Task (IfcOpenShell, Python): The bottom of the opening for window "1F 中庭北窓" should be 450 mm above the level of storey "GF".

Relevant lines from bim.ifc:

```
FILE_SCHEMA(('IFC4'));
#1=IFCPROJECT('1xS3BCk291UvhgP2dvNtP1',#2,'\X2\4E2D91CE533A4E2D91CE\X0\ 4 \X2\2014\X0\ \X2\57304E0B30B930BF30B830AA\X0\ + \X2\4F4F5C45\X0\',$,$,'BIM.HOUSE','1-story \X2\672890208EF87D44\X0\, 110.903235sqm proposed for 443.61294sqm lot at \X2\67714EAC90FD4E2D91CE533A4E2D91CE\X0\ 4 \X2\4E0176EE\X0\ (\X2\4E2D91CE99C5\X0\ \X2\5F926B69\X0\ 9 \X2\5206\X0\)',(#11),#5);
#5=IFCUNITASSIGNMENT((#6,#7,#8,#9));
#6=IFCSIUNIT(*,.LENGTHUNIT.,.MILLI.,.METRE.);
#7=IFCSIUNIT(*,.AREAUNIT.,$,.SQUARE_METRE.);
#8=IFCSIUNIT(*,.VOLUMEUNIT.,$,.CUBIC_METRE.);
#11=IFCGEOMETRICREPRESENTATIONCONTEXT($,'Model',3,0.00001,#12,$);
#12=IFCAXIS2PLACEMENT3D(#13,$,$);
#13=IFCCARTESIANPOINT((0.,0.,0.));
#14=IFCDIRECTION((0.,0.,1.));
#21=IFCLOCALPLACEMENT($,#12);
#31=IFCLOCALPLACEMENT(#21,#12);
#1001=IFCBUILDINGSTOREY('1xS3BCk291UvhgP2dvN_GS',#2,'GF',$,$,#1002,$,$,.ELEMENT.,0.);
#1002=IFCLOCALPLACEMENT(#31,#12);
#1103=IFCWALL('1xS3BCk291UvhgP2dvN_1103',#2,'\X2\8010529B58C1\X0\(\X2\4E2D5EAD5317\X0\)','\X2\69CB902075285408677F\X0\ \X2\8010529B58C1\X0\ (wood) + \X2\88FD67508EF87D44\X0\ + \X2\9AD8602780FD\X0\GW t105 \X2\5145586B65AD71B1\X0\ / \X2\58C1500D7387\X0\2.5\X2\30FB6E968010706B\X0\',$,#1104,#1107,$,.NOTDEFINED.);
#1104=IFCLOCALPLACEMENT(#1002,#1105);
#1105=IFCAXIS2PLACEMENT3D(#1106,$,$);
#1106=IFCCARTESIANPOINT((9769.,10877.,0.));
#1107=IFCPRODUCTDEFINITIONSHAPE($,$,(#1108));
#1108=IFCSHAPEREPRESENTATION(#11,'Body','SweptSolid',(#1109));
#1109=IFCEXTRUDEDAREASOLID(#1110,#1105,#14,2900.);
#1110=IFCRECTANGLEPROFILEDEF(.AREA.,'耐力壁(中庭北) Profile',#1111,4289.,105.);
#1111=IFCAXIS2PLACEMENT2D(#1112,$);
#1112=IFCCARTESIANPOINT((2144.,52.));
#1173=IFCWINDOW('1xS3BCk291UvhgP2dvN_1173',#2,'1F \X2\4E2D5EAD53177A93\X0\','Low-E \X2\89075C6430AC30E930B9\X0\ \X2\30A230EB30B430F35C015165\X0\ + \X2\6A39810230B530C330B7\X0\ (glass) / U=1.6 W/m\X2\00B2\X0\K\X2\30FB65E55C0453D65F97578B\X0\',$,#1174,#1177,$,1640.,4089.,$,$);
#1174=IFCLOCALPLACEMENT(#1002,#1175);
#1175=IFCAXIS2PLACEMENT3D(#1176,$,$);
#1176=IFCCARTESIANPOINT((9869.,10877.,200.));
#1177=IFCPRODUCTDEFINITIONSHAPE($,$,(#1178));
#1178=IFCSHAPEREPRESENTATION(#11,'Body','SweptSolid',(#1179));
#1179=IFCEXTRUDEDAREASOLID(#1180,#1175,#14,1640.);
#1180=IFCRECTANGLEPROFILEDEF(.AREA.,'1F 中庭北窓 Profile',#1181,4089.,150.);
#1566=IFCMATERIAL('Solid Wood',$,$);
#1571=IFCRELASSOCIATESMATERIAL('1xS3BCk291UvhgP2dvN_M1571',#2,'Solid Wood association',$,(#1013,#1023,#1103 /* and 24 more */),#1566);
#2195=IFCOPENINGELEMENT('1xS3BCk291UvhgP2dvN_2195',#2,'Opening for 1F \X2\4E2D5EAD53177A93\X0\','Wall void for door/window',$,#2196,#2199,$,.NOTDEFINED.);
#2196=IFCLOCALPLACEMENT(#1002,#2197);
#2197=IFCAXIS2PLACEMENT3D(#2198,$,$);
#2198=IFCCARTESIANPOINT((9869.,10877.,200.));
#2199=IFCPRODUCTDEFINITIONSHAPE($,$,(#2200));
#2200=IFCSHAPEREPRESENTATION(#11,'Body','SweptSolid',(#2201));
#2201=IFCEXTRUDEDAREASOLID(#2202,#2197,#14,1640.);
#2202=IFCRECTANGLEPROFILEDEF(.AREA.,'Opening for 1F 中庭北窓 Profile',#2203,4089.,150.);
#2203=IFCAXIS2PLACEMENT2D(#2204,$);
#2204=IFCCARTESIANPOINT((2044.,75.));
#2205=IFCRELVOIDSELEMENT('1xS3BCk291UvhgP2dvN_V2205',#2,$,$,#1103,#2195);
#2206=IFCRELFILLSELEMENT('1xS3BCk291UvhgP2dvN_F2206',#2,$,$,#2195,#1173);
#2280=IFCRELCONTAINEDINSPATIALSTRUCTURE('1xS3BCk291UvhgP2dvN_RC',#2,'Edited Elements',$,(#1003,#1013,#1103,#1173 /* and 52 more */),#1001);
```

```python
import numpy as np
import ifcopenshell
import ifcopenshell.api.geometry
import ifcopenshell.geom
import ifcopenshell.util.element
import ifcopenshell.util.placement
import ifcopenshell.util.shape
import ifcopenshell.util.unit

model = ifcopenshell.open("bim.ifc")
unit_scale = ifcopenshell.util.unit.calculate_unit_scale(model)

window = model.by_id(1173)
opening = window.FillsVoids[0].RelatingOpeningElement
storey = ifcopenshell.util.element.get_container(window, ifc_class="IfcBuildingStorey")
level = ifcopenshell.util.placement.get_local_placement(storey.ObjectPlacement)[2, 3]

# The opening's origin need not be at the sill, so measure its lowest point.
shape = ifcopenshell.geom.create_shape(ifcopenshell.geom.settings(), opening)
bottom = ifcopenshell.util.shape.get_shape_bottom_elevation(shape, shape.geometry) / unit_scale
dz = level + 0.45 / unit_scale - bottom

shift = np.array([0.0, 0.0, dz])
# The window is not placed relative to its opening, so move both.
for product in (opening, window):
    matrix = ifcopenshell.util.placement.get_local_placement(product.ObjectPlacement)
    matrix[:3, 3] += shift
    ifcopenshell.api.geometry.edit_object_placement(model, product=product, matrix=matrix, is_si=False)

print(f"moved by {dz * unit_scale:+.3f} m")

model.write("bim_v2.ifc")
```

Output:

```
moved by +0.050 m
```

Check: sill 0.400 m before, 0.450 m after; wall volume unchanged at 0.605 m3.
